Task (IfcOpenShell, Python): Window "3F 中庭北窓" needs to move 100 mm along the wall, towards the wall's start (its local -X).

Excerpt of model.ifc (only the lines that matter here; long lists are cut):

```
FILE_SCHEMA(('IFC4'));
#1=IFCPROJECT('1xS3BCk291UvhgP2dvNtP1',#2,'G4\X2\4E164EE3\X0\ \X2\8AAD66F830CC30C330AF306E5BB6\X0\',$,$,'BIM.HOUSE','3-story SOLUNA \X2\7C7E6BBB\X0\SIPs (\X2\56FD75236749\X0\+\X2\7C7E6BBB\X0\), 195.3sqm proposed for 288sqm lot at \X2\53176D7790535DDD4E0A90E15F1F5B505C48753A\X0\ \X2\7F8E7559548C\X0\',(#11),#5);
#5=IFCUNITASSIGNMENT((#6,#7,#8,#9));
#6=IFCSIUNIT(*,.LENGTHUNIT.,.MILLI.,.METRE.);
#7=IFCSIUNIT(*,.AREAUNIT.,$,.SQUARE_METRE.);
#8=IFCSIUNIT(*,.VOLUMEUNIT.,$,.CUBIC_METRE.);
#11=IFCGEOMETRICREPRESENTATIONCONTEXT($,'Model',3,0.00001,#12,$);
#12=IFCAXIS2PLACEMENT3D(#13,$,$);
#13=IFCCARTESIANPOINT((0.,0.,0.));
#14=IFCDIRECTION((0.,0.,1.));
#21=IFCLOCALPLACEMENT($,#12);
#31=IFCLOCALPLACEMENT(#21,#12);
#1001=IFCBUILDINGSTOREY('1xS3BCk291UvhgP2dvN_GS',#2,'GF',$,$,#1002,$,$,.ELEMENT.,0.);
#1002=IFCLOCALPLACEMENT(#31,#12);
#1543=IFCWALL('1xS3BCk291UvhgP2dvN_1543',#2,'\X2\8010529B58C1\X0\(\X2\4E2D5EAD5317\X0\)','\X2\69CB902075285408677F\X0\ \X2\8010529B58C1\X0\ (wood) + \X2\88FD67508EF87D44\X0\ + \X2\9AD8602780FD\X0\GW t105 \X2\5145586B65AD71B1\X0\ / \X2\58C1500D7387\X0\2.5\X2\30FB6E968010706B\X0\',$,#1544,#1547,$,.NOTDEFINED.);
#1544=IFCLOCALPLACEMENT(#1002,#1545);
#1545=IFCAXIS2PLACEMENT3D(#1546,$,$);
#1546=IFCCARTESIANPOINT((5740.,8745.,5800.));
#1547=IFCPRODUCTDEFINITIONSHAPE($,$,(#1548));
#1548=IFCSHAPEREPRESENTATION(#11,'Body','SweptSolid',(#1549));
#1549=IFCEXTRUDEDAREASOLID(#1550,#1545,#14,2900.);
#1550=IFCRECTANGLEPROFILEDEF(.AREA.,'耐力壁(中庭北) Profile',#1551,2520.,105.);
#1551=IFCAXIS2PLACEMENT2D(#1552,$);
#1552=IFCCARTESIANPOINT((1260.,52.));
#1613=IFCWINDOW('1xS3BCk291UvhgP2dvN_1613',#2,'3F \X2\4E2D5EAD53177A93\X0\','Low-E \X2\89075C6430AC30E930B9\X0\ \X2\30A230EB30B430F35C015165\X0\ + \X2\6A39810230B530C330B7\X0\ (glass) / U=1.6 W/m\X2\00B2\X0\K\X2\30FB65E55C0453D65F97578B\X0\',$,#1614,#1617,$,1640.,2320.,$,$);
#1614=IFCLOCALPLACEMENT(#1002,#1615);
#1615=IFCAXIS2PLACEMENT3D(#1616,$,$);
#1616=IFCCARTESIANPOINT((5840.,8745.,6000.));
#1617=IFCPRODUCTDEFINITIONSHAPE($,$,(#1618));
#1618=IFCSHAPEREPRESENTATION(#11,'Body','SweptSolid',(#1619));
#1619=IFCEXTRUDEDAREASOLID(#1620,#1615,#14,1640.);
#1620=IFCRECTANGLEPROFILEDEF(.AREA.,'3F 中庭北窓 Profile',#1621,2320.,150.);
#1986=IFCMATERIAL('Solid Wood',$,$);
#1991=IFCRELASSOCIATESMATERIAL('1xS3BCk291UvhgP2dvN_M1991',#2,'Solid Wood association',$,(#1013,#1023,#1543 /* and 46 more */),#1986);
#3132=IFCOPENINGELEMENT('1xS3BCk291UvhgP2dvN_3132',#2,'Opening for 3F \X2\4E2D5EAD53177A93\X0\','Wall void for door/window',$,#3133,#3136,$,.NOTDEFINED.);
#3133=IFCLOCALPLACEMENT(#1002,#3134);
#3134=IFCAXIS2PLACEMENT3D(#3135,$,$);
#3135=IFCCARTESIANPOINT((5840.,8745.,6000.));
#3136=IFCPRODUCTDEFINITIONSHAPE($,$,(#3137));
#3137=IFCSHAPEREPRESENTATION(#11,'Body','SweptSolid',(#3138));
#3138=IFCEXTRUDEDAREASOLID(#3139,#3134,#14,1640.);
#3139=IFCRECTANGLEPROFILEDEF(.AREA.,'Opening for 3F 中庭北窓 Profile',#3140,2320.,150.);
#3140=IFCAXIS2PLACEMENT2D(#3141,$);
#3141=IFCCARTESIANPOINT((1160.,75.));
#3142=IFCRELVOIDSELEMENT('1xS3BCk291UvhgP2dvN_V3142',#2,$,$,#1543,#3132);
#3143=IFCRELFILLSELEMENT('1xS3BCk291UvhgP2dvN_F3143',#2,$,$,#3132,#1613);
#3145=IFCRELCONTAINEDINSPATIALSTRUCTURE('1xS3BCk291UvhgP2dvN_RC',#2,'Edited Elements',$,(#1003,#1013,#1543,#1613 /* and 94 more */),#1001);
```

```python
import ifcopenshell
import ifcopenshell.api.geometry
import ifcopenshell.util.placement

model = ifcopenshell.open("model.ifc")

window = model.by_id(1613)
opening = window.FillsVoids[0].RelatingOpeningElement
wall = opening.VoidsElements[0].RelatingBuildingElement

wall_matrix = ifcopenshell.util.placement.get_local_placement(wall.ObjectPlacement)
shift = wall_matrix[:3, 0] * -100.0
before = ifcopenshell.util.placement.get_local_placement(window.ObjectPlacement)[:3, 3].copy()

# The window is not placed relative to its opening, so move both.
for product in (opening, window):
    matrix = ifcopenshell.util.placement.get_local_placement(product.ObjectPlacement)
    matrix[:3, 3] += shift
    ifcopenshell.api.geometry.edit_object_placement(model, product=product, matrix=matrix, is_si=False)

after = ifcopenshell.util.placement.get_local_placement(window.ObjectPlacement)[:3, 3]
print("window moved by", (after - before).round(3) + 0.0)

model.write("model_updated.ifc")
```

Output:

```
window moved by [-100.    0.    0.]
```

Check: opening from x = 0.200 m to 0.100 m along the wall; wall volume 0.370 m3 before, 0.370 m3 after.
